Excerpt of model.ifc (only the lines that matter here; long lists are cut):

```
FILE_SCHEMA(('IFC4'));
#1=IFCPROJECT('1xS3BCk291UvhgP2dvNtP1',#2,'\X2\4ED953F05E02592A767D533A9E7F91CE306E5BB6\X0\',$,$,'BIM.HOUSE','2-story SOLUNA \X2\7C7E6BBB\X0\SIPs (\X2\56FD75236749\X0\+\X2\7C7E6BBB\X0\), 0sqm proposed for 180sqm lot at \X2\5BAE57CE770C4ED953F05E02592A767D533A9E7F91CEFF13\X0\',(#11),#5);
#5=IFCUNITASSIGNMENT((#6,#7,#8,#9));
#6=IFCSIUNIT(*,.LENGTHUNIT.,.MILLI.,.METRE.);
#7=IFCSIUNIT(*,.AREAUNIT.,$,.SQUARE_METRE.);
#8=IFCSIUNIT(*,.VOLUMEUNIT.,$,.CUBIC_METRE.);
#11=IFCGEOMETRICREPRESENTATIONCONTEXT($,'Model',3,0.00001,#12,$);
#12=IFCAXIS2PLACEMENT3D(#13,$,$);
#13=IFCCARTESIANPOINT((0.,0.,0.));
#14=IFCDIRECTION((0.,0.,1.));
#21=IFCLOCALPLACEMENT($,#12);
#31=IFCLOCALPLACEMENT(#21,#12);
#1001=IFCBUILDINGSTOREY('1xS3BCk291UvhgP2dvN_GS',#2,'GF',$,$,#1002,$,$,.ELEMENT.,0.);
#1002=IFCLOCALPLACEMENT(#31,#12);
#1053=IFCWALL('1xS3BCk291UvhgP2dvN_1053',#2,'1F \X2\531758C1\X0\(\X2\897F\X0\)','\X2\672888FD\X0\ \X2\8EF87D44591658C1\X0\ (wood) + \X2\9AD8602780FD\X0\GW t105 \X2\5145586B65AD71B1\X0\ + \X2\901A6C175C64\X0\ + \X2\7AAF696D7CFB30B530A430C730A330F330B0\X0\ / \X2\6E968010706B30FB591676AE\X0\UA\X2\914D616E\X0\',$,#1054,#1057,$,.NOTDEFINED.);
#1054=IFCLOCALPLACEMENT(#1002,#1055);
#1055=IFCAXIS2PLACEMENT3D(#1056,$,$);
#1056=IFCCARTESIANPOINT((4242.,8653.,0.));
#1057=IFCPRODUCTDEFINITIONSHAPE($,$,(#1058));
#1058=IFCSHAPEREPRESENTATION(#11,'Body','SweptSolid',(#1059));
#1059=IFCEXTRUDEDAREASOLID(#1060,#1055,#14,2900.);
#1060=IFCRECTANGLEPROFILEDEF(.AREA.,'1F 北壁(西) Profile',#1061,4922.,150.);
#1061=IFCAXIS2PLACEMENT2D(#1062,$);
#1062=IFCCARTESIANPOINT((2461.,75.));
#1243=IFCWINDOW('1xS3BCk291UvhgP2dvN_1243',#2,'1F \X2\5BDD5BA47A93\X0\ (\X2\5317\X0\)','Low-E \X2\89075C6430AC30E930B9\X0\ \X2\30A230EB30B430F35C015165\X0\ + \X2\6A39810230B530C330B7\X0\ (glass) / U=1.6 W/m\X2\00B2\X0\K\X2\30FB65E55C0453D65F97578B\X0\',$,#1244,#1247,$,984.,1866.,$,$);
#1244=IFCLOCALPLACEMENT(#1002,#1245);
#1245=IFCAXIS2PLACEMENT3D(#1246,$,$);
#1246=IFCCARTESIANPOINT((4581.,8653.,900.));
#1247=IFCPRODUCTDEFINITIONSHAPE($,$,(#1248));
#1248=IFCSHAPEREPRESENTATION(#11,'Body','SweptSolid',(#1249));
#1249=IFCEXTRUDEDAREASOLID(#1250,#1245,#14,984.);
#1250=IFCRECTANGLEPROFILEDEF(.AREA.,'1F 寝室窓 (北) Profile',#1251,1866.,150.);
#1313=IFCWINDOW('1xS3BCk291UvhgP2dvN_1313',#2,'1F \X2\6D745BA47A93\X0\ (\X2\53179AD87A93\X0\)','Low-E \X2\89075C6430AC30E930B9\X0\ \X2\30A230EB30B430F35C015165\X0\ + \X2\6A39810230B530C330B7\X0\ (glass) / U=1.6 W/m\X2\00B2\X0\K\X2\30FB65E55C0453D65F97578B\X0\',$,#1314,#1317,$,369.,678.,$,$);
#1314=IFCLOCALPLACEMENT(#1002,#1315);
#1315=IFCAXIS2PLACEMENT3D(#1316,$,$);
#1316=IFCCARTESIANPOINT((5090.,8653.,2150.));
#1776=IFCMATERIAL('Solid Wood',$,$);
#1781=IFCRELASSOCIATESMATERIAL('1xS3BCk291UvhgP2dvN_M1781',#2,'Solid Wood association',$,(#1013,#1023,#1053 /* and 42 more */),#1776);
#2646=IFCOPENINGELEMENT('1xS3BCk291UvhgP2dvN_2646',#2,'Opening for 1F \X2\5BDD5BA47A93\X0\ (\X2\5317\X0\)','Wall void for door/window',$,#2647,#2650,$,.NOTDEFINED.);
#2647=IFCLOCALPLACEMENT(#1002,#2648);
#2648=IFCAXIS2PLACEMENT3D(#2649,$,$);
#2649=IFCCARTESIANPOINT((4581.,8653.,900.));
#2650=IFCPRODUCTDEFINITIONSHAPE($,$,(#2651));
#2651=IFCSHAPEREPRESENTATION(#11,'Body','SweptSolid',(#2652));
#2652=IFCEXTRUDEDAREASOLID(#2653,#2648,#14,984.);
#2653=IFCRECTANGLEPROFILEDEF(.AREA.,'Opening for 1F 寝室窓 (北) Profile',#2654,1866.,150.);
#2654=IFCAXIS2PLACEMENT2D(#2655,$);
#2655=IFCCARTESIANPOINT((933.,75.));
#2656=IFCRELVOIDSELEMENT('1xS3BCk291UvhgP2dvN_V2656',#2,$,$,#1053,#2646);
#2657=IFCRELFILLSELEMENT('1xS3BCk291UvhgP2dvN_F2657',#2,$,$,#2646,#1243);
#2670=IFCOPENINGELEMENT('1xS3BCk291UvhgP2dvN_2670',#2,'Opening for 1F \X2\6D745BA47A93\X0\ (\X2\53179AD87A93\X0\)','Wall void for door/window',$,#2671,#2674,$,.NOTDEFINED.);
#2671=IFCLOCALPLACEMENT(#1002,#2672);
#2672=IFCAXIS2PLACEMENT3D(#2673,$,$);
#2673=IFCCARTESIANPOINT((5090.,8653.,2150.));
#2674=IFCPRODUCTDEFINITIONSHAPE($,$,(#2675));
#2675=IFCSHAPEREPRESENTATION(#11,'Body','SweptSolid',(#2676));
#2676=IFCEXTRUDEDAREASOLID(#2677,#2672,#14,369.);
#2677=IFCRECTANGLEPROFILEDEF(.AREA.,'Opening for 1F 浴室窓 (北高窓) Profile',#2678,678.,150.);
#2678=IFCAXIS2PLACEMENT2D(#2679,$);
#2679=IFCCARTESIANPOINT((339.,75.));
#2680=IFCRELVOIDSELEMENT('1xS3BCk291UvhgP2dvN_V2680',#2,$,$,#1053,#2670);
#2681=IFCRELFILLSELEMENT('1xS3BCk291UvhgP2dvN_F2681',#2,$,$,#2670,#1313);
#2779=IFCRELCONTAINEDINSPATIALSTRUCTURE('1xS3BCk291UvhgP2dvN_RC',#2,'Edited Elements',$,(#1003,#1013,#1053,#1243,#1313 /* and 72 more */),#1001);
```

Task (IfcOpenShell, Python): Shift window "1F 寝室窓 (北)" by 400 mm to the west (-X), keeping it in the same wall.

```python
import ifcopenshell
import ifcopenshell.api.geometry
import ifcopenshell.util.placement

model = ifcopenshell.open("model.ifc")

window = model.by_guid("1xS3BCk291UvhgP2dvN_1243")
opening = window.FillsVoids[0].RelatingOpeningElement
wall = opening.VoidsElements[0].RelatingBuildingElement

wall_matrix = ifcopenshell.util.placement.get_local_placement(wall.ObjectPlacement)
shift = wall_matrix[:3, 0] * -400.0
before = ifcopenshell.util.placement.get_local_placement(window.ObjectPlacement)[:3, 3].copy()

# The window is not placed relative to its opening, so move both.
for product in (opening, window):
    matrix = ifcopenshell.util.placement.get_local_placement(product.ObjectPlacement)
    matrix[:3, 3] += shift
    ifcopenshell.api.geometry.edit_object_placement(model, product=product, matrix=matrix, is_si=False)

after = ifcopenshell.util.placement.get_local_placement(window.ObjectPlacement)[:3, 3]
print("window moved by", (after - before).round(3) + 0.0)

model.write("model_edited.ifc")
```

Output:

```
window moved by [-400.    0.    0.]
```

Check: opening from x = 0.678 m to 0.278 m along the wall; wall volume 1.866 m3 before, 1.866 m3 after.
